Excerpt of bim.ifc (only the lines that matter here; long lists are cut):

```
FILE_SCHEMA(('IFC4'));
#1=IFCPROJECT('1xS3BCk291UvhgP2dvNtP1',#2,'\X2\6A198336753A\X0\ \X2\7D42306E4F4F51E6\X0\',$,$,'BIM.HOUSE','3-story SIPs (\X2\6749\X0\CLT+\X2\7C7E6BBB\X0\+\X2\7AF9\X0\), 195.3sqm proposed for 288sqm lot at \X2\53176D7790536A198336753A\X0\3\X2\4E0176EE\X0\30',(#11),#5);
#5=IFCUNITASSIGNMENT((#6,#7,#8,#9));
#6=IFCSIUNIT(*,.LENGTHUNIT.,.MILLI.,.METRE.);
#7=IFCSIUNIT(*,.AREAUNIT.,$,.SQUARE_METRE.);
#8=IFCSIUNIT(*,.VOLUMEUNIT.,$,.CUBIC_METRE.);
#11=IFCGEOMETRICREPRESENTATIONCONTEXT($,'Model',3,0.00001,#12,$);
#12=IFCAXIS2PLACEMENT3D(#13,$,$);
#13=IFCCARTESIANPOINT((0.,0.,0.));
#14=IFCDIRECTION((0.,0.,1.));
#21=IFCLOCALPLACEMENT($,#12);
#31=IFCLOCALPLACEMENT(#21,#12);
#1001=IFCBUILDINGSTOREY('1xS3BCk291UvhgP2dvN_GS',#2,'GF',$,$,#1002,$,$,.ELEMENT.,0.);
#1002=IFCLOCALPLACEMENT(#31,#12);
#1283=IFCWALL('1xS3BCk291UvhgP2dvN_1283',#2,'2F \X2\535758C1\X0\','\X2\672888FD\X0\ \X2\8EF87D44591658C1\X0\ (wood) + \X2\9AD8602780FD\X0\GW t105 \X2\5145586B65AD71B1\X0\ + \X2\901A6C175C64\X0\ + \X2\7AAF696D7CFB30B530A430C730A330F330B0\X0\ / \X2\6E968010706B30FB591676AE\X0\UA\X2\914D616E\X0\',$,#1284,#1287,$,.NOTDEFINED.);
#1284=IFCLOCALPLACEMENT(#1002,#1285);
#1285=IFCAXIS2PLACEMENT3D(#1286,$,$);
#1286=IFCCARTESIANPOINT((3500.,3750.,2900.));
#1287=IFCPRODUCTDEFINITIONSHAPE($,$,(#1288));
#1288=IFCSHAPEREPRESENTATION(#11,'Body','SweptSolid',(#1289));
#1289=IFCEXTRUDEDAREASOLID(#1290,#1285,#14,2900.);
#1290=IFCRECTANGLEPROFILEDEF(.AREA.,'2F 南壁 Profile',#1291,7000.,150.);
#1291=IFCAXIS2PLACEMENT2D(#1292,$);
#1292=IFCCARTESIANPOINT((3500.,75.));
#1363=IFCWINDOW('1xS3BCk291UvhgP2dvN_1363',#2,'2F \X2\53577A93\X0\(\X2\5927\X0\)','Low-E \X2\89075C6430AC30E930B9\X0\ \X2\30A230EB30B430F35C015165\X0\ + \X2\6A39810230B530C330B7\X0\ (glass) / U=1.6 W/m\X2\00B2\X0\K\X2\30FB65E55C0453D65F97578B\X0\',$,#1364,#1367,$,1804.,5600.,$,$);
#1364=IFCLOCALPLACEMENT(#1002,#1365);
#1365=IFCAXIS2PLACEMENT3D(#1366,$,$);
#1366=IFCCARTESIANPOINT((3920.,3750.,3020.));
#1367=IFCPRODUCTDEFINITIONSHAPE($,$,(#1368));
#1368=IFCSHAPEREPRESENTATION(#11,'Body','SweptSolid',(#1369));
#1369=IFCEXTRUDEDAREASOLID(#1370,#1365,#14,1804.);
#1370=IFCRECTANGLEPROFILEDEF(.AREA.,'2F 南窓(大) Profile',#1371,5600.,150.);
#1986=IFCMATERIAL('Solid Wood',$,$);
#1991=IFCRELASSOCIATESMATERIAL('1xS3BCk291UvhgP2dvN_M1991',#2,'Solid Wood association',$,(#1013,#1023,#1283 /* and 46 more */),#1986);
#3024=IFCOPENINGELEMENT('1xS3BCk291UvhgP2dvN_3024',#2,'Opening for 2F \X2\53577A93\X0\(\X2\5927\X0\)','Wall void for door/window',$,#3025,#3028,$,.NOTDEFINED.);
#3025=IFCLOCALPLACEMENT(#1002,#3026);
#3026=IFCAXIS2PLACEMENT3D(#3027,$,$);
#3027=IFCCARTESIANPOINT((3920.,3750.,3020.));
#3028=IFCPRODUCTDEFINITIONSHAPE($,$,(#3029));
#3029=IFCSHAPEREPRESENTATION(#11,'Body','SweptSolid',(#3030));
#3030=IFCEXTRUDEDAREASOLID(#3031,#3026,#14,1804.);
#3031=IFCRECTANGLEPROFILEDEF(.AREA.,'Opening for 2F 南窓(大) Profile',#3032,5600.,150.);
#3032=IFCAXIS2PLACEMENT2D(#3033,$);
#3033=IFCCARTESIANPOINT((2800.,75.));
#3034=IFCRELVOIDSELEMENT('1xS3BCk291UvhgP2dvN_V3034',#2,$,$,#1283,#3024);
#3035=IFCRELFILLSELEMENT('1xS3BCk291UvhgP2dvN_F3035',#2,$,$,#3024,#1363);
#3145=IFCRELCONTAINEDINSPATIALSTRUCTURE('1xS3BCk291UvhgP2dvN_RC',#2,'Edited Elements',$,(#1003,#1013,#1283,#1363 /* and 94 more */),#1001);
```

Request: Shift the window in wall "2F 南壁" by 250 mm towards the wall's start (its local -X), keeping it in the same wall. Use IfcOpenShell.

```python
import ifcopenshell
import ifcopenshell.api.geometry
import ifcopenshell.util.placement

model = ifcopenshell.open("bim.ifc")

window = model.by_guid("1xS3BCk291UvhgP2dvN_1363")
opening = window.FillsVoids[0].RelatingOpeningElement
wall = opening.VoidsElements[0].RelatingBuildingElement

wall_matrix = ifcopenshell.util.placement.get_local_placement(wall.ObjectPlacement)
shift = wall_matrix[:3, 0] * -250.0
before = ifcopenshell.util.placement.get_local_placement(window.ObjectPlacement)[:3, 3].copy()

# The window is not placed relative to its opening, so move both.
for product in (opening, window):
    matrix = ifcopenshell.util.placement.get_local_placement(product.ObjectPlacement)
    matrix[:3, 3] += shift
    ifcopenshell.api.geometry.edit_object_placement(model, product=product, matrix=matrix, is_si=False)

after = ifcopenshell.util.placement.get_local_placement(window.ObjectPlacement)[:3, 3]
print("window moved by", (after - before).round(3) + 0.0)

model.write("bim_edited.ifc")
```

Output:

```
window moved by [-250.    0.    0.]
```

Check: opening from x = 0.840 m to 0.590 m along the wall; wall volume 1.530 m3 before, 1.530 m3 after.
